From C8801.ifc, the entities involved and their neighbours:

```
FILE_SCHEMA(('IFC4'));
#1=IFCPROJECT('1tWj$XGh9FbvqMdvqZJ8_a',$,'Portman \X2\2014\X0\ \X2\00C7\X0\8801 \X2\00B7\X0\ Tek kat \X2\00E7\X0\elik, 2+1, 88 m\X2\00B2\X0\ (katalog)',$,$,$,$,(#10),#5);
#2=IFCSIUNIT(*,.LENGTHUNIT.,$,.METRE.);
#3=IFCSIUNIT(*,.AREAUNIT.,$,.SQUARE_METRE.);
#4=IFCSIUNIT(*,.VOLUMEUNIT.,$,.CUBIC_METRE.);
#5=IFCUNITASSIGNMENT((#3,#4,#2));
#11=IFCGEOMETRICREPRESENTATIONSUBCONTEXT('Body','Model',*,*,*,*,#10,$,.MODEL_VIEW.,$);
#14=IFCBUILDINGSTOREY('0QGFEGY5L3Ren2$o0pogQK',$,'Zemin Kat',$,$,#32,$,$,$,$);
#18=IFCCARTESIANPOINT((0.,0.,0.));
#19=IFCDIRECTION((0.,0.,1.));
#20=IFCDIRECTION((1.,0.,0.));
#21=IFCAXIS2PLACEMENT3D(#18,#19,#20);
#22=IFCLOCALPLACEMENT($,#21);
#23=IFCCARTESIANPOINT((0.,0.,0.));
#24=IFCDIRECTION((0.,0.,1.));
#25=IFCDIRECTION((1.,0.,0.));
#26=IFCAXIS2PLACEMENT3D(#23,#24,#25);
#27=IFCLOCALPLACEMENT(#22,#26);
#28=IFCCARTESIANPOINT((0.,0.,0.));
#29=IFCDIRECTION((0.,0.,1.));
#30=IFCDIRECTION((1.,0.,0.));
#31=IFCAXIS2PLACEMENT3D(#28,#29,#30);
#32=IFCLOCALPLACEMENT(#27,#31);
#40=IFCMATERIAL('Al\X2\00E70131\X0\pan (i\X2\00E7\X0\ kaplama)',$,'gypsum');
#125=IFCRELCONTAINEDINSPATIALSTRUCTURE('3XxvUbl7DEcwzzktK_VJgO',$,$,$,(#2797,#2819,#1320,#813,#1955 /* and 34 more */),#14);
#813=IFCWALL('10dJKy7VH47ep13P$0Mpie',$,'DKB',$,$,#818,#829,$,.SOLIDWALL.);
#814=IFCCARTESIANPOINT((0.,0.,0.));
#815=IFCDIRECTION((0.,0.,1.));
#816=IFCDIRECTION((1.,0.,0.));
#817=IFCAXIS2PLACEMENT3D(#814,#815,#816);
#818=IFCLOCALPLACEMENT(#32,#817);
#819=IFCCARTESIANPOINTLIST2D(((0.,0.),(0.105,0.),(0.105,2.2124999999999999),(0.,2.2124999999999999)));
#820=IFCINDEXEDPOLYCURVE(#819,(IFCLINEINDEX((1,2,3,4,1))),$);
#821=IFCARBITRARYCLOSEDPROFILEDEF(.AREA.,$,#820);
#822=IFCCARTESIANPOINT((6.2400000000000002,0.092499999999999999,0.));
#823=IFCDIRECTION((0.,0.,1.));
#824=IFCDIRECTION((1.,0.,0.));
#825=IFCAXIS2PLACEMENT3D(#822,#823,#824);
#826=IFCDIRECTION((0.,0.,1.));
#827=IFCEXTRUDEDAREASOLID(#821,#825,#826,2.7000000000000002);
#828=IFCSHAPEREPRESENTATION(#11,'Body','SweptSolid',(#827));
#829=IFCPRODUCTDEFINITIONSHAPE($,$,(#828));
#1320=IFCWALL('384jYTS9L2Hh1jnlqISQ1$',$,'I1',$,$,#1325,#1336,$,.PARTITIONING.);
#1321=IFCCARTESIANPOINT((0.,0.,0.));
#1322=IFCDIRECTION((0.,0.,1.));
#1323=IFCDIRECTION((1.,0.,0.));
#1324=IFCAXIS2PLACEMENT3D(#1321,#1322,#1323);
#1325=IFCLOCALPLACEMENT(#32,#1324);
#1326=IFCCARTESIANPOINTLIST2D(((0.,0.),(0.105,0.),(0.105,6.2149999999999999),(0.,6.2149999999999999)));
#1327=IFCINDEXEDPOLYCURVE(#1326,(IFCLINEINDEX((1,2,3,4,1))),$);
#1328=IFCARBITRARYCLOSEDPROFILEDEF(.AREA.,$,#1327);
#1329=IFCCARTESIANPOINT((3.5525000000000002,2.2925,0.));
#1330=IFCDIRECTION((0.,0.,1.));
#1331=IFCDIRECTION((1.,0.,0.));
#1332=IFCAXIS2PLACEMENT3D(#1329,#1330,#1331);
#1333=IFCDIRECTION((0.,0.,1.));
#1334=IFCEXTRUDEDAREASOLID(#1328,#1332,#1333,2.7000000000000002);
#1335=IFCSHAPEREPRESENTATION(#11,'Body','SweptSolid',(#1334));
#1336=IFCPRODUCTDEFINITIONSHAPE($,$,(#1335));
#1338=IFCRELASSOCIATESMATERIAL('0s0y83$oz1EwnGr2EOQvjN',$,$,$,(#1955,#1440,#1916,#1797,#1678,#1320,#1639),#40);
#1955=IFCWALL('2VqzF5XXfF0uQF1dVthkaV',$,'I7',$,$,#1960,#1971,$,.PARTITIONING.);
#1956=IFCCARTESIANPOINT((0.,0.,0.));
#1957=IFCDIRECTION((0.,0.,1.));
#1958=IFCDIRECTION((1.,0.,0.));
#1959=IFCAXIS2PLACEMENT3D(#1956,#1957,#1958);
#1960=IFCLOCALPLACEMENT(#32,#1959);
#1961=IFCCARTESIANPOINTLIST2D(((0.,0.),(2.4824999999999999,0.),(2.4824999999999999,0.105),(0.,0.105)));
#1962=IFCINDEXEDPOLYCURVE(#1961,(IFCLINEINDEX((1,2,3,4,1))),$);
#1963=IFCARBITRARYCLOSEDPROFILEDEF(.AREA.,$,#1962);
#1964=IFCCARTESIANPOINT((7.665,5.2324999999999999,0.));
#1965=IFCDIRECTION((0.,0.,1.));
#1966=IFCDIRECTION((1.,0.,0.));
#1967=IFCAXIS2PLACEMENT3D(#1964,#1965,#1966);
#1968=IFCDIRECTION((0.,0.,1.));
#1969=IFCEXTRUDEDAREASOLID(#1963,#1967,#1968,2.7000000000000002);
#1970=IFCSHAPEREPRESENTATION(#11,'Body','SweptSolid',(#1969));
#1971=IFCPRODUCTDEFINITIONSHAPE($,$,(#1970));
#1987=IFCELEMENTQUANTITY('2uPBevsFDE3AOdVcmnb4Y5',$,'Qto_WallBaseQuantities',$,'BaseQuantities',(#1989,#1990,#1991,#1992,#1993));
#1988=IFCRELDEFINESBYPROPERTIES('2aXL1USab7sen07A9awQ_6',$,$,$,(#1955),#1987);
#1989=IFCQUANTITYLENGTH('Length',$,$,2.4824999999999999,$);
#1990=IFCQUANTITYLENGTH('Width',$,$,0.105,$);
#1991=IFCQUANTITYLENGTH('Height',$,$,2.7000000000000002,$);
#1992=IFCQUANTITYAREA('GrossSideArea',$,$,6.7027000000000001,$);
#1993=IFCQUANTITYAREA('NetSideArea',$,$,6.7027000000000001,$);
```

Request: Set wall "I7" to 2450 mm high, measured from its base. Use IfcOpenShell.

```python
import ifcopenshell
import ifcopenshell.api.pset
import ifcopenshell.geom
import ifcopenshell.util.element
import ifcopenshell.util.representation
import ifcopenshell.util.shape
import ifcopenshell.util.unit

model = ifcopenshell.open("C8801.ifc")
unit_scale = ifcopenshell.util.unit.calculate_unit_scale(model)
area_scale = ifcopenshell.util.unit.calculate_unit_scale(model, "AREAUNIT")
settings = ifcopenshell.geom.settings()


def volume(element):
    """Net volume in cubic metres, openings subtracted."""
    shape = ifcopenshell.geom.create_shape(settings, element)
    return ifcopenshell.util.shape.get_volume(shape.geometry)


wall = model.by_id(1955)
before = volume(wall)

body = ifcopenshell.util.representation.get_representation(wall, "Model", "Body")
solid = body.Items[0]
old_height = solid.Depth
solid.Depth = 2.45 / unit_scale
after = volume(wall)
thickness = 0.105  # wall thickness in metres

# Update the stored height, areas and volumes.
qto = model.by_id(ifcopenshell.util.element.get_pset(wall, "Qto_WallBaseQuantities", should_inherit=False)["id"])
ifcopenshell.api.pset.edit_qto(model, qto=qto, properties={
    "Height": solid.Depth,
    "GrossSideArea": ifcopenshell.util.element.get_pset(wall, "Qto_WallBaseQuantities", "GrossSideArea") * solid.Depth / old_height,
    "NetSideArea": after / thickness / area_scale,
})

print(f"height {old_height:g} -> {solid.Depth:g}, volume {before:.3f} -> {after:.3f} m3")

model.write("C8801-out.ifc")
```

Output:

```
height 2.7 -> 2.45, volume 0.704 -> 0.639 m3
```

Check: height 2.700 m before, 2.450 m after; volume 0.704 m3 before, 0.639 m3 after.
